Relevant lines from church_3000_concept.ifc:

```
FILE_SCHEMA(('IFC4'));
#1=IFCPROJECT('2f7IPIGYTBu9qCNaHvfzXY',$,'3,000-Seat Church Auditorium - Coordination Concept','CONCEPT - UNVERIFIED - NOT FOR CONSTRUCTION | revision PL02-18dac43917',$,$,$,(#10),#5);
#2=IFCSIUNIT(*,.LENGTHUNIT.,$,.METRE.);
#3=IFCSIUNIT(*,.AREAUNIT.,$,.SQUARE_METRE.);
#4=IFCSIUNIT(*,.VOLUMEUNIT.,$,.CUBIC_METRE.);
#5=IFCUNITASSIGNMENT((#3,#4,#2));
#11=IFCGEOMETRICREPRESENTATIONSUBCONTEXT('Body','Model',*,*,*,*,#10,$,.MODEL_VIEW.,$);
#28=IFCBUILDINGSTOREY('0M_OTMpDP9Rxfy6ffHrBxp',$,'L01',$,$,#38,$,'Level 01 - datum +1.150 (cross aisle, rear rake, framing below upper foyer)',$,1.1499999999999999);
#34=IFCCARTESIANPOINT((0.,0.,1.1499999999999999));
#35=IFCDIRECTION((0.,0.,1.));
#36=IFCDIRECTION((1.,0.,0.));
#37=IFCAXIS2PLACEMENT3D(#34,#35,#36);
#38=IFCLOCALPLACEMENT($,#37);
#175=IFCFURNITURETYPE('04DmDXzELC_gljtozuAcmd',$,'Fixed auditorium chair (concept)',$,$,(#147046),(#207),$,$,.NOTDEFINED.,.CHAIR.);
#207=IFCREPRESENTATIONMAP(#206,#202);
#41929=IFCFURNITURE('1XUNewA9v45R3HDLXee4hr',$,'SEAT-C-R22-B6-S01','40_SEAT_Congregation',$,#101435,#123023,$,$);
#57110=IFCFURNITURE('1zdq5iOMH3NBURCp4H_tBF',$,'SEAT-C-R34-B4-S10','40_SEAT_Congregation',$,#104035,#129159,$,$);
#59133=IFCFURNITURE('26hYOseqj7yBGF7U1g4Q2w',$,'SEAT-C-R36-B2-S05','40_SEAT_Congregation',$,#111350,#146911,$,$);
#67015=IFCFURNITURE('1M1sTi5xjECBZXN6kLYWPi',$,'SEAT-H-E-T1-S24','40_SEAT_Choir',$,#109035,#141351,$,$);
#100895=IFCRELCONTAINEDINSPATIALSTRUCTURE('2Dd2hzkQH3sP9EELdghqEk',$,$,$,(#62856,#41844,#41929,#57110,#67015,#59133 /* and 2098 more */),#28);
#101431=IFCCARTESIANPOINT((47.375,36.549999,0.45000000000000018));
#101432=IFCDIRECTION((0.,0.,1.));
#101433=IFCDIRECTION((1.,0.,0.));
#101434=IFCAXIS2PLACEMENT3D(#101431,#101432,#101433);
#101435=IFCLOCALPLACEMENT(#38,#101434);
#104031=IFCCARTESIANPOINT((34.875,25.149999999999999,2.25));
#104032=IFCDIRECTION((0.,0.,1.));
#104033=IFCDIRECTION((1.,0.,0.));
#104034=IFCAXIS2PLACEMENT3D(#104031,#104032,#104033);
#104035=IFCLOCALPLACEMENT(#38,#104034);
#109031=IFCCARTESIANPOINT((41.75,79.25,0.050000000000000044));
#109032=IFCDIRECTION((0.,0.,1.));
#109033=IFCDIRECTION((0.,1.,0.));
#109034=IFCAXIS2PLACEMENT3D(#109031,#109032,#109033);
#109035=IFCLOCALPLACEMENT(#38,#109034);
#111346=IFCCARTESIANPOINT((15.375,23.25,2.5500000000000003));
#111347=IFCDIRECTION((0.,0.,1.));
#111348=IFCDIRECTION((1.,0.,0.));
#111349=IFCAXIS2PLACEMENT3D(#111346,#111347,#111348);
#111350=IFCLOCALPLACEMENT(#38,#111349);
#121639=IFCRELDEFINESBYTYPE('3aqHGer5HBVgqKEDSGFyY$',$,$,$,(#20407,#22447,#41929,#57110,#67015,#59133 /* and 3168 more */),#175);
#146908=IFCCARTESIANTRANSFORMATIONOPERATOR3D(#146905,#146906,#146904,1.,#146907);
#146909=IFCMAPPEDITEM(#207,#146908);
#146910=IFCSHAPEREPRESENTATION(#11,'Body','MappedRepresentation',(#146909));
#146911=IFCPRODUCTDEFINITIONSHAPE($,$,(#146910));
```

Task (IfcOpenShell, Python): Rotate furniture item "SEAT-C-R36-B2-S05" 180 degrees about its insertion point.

```python
import ifcopenshell
import ifcopenshell.api.geometry
import ifcopenshell.util.placement

model = ifcopenshell.open("church_3000_concept.ifc")

item = model.by_guid("26hYOseqj7yBGF7U1g4Q2w")
matrix = ifcopenshell.util.placement.get_local_placement(item.ObjectPlacement)
matrix = matrix @ ifcopenshell.util.placement.rotation(180, "Z")
ifcopenshell.api.geometry.edit_object_placement(model, product=item, matrix=matrix, is_si=False)

print(ifcopenshell.util.placement.get_local_placement(item.ObjectPlacement).round(3) + 0.0)

model.write("church_3000_concept_v2.ifc")
```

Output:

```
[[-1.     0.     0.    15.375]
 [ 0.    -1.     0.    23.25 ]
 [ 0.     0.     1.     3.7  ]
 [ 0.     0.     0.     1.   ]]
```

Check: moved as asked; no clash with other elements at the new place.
